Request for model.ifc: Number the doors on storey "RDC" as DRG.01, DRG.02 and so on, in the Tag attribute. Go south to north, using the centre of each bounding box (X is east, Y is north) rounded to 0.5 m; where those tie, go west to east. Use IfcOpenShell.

First a look at what the model holds.

```python
import ifcopenshell
import ifcopenshell.util.element
import ifcopenshell.util.placement

model = ifcopenshell.open("model.ifc")
print(model.schema)
storey = next(s for s in model.by_type("IfcBuildingStorey") if s.Name == "RDC")
doors = [e for e in ifcopenshell.util.element.get_decomposition(storey) if e.is_a("IfcDoor")]
for e in sorted(doors, key=lambda e: e.id()):
    origin = ifcopenshell.util.placement.get_local_placement(e.ObjectPlacement)[:3, 3]
    print(e.id(), e.Tag, e.Name, origin.round(2) + 0.0, sep=" | ")
```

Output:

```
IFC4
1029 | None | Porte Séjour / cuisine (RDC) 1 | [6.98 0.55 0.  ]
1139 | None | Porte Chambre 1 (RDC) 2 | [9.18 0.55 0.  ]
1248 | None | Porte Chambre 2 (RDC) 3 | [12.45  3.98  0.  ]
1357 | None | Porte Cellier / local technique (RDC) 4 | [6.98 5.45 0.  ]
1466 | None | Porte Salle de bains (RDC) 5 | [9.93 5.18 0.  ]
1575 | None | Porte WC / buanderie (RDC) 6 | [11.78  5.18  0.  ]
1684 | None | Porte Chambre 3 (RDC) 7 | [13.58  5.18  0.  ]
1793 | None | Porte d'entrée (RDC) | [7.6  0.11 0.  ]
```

```python
import ifcopenshell
import ifcopenshell.geom
import ifcopenshell.util.element
import ifcopenshell.util.shape

model = ifcopenshell.open("model.ifc")
settings = ifcopenshell.geom.settings()
settings.set("use-world-coords", True)


def centre(element):
    shape = ifcopenshell.geom.create_shape(settings, element)
    return ifcopenshell.util.shape.get_bbox_centroid(shape.geometry)


storey = next(s for s in model.by_type("IfcBuildingStorey") if s.Name == "RDC")
doors = [e for e in ifcopenshell.util.element.get_decomposition(storey) if e.is_a("IfcDoor")]

# Insertion points can sit at a corner or the storey origin, so sort by the geometry (in metres).
centres = {e: centre(e) for e in doors}
doors.sort(key=lambda e: (round(centres[e][1] / 0.5), centres[e][0]))

for i, e in enumerate(doors, start=1):
    number = f"DRG.{i:02d}"
    e.Tag = number
    print(e.id(), number)

model.write("model_v2.ifc")
```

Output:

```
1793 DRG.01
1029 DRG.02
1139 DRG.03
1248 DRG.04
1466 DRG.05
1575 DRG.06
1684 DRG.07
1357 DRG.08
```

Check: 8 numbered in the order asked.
